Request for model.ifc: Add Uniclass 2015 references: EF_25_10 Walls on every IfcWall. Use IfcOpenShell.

First a look at what the model holds.

```python
import ifcopenshell

model = ifcopenshell.open("model.ifc")
print(model.schema)
print("classifications:", [c.Name for c in model.by_type("IfcClassification")])
for ifc_class in ("IfcDoor", "IfcRoof", "IfcStair", "IfcWall", "IfcWindow"):
    print(ifc_class, len(model.by_type(ifc_class)))
```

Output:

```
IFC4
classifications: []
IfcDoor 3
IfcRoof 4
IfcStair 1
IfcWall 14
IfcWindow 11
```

```python
import ifcopenshell
import ifcopenshell.api.classification

model = ifcopenshell.open("model.ifc")

system = ifcopenshell.api.classification.add_classification(model, classification="Uniclass 2015")

codes = {
    "IfcWall": ("EF_25_10", "Walls"),
}
for ifc_class, (code, name) in codes.items():
    products = model.by_type(ifc_class)
    ifcopenshell.api.classification.add_reference(
        model, products=products, classification=system, identification=code, name=name
    )
    print(code, len(products))

model.write("model_v2.ifc")
```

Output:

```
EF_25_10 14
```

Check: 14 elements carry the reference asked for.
